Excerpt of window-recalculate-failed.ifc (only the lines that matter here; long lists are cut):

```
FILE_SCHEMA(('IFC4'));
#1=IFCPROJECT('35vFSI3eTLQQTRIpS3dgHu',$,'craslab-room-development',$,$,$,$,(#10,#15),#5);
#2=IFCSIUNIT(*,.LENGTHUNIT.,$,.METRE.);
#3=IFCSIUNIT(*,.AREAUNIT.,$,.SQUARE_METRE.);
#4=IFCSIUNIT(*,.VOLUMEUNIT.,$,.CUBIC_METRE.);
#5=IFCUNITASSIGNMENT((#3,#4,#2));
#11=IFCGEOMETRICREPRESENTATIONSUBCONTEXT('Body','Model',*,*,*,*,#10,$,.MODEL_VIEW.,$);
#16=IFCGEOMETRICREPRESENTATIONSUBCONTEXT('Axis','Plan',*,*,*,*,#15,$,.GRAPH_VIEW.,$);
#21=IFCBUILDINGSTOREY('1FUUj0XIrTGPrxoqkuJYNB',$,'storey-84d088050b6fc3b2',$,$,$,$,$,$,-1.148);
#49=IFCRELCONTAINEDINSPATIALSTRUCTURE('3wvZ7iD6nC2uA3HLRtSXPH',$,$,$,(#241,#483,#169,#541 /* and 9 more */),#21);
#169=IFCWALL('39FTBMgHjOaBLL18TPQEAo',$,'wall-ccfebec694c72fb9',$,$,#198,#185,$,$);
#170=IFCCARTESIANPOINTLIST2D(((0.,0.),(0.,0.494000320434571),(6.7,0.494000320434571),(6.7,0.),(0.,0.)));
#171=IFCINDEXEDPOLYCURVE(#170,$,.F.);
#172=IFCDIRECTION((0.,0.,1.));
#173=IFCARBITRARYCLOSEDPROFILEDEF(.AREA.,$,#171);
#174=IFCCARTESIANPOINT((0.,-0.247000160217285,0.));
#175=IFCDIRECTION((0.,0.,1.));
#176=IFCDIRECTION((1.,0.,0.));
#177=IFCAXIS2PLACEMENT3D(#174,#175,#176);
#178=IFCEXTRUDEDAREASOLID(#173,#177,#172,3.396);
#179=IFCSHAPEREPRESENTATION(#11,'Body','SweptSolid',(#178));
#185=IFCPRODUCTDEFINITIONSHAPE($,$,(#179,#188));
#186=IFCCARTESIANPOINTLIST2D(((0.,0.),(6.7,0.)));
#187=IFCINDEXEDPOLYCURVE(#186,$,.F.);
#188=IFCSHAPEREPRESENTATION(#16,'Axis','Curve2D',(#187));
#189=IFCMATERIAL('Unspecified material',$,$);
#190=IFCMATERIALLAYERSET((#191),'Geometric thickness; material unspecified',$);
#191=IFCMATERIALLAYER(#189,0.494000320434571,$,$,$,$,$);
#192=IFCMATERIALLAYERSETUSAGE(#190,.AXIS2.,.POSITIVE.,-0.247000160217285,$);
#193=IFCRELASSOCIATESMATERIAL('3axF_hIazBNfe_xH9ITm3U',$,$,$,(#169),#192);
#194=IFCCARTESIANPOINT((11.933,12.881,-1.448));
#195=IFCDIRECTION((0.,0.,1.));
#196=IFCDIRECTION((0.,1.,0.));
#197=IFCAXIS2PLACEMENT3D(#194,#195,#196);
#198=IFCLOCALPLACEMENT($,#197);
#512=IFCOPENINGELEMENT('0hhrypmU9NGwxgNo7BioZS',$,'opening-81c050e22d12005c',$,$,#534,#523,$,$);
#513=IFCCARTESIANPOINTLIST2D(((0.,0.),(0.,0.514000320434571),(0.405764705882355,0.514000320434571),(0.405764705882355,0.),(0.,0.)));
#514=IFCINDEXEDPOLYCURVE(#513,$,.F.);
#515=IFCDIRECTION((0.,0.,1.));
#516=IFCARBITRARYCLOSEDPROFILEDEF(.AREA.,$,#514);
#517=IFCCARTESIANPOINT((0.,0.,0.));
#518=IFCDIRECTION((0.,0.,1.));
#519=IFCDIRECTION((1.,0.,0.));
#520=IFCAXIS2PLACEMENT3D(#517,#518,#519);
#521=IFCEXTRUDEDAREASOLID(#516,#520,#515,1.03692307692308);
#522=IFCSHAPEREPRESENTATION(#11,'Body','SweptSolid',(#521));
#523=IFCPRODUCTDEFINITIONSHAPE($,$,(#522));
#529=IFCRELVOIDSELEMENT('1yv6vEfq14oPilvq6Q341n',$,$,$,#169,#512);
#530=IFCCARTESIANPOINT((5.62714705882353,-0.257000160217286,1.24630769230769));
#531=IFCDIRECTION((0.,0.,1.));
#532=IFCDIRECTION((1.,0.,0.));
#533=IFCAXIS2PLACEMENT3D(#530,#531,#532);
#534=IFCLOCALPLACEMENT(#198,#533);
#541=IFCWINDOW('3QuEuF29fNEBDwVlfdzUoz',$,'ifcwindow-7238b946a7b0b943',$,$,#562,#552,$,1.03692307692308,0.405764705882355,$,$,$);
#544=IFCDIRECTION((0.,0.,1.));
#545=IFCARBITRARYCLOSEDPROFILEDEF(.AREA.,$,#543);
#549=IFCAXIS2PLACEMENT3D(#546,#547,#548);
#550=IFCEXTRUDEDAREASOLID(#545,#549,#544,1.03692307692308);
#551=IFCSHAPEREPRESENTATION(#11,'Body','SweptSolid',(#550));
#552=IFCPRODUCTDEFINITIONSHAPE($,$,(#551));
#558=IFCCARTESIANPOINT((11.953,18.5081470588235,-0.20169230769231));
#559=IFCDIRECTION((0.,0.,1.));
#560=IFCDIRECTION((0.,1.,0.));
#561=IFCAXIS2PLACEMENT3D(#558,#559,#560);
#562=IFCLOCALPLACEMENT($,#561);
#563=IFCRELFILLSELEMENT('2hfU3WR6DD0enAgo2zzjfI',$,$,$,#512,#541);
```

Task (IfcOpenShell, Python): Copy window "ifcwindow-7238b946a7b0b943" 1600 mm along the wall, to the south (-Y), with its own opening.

```python
import ifcopenshell
import ifcopenshell.api.feature
import ifcopenshell.api.geometry
import ifcopenshell.api.root
import ifcopenshell.geom
import ifcopenshell.util.element
import ifcopenshell.util.placement
import ifcopenshell.util.shape

model = ifcopenshell.open("window-recalculate-failed.ifc")
settings = ifcopenshell.geom.settings()


def volume(element):
    """Net volume in cubic metres, openings subtracted."""
    shape = ifcopenshell.geom.create_shape(settings, element)
    return ifcopenshell.util.shape.get_volume(shape.geometry)


window = model.by_guid("3QuEuF29fNEBDwVlfdzUoz")
opening = window.FillsVoids[0].RelatingOpeningElement
wall = opening.VoidsElements[0].RelatingBuildingElement
before = volume(wall)
shift = ifcopenshell.util.placement.get_local_placement(wall.ObjectPlacement)[:3, 0] * -1.6

# copy_class copies the void relationship, type, container and properties, but no geometry.
new_opening = ifcopenshell.api.root.copy_class(model, product=opening)
new_opening.Representation = ifcopenshell.util.element.copy_deep(
    model, opening.Representation, exclude=["IfcGeometricRepresentationContext", "IfcRepresentationMap"]
)
new_window = ifcopenshell.api.root.copy_class(model, product=window)
new_window.Representation = ifcopenshell.util.element.copy_deep(
    model, window.Representation, exclude=["IfcGeometricRepresentationContext", "IfcRepresentationMap"]
)
ifcopenshell.api.feature.add_filling(model, opening=new_opening, element=new_window)

for old, new in ((opening, new_opening), (window, new_window)):
    matrix = ifcopenshell.util.placement.get_local_placement(old.ObjectPlacement)
    matrix[:3, 3] += shift
    ifcopenshell.api.geometry.edit_object_placement(model, product=new, matrix=matrix, is_si=False)

after = volume(wall)

print(f"wall volume {before:.3f} -> {after:.3f} m3")

model.write("window-recalculate-failed_updated.ifc")
```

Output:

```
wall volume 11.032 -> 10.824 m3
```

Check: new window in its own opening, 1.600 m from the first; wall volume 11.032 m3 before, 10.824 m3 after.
